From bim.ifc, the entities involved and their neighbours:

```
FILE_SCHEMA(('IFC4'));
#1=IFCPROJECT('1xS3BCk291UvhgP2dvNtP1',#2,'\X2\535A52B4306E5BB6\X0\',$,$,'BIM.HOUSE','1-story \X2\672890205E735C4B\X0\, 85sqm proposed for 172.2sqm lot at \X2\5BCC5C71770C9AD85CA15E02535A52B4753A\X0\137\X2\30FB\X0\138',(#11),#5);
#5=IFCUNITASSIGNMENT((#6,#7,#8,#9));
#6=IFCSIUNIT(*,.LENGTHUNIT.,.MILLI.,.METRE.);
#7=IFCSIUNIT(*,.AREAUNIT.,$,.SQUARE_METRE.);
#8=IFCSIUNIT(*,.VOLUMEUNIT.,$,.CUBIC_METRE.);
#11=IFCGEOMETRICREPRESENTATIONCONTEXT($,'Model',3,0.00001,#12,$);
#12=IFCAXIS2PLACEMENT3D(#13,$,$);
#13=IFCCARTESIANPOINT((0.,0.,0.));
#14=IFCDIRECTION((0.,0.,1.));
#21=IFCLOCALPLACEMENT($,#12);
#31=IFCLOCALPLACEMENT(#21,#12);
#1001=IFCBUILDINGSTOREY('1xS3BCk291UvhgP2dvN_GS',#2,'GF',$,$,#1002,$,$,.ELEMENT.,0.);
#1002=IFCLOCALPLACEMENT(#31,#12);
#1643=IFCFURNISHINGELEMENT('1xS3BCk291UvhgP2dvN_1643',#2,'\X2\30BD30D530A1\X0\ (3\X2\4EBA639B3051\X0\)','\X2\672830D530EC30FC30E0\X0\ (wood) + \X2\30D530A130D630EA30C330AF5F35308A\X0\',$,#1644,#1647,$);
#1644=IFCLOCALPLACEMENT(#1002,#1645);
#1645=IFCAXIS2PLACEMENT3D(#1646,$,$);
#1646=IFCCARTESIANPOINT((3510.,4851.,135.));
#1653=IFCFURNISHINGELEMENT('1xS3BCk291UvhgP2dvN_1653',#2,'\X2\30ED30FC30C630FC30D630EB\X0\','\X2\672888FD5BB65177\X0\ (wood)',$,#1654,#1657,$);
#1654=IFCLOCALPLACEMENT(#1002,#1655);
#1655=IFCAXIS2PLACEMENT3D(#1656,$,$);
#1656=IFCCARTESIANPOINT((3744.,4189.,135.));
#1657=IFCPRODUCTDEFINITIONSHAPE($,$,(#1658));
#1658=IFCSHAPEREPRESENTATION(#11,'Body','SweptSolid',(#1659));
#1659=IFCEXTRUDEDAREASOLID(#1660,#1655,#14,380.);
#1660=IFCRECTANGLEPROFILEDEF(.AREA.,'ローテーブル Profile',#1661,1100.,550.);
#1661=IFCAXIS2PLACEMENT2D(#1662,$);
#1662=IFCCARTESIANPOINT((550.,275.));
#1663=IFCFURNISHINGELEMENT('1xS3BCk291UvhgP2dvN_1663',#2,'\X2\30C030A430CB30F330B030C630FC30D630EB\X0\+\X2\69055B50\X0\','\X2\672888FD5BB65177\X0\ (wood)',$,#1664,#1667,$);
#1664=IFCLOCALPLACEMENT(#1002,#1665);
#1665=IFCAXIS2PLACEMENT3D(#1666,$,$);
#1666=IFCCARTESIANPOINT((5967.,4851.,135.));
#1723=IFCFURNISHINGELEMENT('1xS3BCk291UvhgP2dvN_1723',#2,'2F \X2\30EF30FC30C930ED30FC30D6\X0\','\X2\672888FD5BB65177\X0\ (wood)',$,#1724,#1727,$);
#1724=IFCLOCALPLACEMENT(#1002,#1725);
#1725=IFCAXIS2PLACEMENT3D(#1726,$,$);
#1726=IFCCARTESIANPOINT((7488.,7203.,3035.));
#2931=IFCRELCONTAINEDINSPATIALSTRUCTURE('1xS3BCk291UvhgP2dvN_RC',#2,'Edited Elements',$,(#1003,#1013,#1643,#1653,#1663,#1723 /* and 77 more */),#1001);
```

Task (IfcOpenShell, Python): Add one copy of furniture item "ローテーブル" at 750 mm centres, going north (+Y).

```python
import numpy as np
import ifcopenshell
import ifcopenshell.api.geometry
import ifcopenshell.api.root
import ifcopenshell.util.element
import ifcopenshell.util.placement

model = ifcopenshell.open("bim.ifc")


def reuse_history(source, copy):
    """copy_class also copies each property set's owner history, people and application; keep the originals."""
    for rel in copy.IsDefinedBy:
        if rel.is_a("IfcRelDefinesByProperties") and (history := rel.RelatingPropertyDefinition.OwnerHistory):
            rel.RelatingPropertyDefinition.OwnerHistory = source.OwnerHistory
            ifcopenshell.util.element.remove_deep2(model, history)


source = model.by_id(1653)
base = ifcopenshell.util.placement.get_local_placement(source.ObjectPlacement)
step = np.array([0.0, 1.0, 0.0]) * 750.0

for i in range(1, 2):
    copy = ifcopenshell.api.root.copy_class(model, product=source)
    copy.Representation = ifcopenshell.util.element.copy_deep(
        model, source.Representation, exclude=["IfcGeometricRepresentationContext", "IfcRepresentationMap"]
    )
    reuse_history(source, copy)
    matrix = base.copy()
    matrix[:3, 3] += i * step
    print("added at", matrix[:3, 3].round(3) + 0.0)
    ifcopenshell.api.geometry.edit_object_placement(model, product=copy, matrix=matrix, is_si=False)

model.write("bim_v2.ifc")
```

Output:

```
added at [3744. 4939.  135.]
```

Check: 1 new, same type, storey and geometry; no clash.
